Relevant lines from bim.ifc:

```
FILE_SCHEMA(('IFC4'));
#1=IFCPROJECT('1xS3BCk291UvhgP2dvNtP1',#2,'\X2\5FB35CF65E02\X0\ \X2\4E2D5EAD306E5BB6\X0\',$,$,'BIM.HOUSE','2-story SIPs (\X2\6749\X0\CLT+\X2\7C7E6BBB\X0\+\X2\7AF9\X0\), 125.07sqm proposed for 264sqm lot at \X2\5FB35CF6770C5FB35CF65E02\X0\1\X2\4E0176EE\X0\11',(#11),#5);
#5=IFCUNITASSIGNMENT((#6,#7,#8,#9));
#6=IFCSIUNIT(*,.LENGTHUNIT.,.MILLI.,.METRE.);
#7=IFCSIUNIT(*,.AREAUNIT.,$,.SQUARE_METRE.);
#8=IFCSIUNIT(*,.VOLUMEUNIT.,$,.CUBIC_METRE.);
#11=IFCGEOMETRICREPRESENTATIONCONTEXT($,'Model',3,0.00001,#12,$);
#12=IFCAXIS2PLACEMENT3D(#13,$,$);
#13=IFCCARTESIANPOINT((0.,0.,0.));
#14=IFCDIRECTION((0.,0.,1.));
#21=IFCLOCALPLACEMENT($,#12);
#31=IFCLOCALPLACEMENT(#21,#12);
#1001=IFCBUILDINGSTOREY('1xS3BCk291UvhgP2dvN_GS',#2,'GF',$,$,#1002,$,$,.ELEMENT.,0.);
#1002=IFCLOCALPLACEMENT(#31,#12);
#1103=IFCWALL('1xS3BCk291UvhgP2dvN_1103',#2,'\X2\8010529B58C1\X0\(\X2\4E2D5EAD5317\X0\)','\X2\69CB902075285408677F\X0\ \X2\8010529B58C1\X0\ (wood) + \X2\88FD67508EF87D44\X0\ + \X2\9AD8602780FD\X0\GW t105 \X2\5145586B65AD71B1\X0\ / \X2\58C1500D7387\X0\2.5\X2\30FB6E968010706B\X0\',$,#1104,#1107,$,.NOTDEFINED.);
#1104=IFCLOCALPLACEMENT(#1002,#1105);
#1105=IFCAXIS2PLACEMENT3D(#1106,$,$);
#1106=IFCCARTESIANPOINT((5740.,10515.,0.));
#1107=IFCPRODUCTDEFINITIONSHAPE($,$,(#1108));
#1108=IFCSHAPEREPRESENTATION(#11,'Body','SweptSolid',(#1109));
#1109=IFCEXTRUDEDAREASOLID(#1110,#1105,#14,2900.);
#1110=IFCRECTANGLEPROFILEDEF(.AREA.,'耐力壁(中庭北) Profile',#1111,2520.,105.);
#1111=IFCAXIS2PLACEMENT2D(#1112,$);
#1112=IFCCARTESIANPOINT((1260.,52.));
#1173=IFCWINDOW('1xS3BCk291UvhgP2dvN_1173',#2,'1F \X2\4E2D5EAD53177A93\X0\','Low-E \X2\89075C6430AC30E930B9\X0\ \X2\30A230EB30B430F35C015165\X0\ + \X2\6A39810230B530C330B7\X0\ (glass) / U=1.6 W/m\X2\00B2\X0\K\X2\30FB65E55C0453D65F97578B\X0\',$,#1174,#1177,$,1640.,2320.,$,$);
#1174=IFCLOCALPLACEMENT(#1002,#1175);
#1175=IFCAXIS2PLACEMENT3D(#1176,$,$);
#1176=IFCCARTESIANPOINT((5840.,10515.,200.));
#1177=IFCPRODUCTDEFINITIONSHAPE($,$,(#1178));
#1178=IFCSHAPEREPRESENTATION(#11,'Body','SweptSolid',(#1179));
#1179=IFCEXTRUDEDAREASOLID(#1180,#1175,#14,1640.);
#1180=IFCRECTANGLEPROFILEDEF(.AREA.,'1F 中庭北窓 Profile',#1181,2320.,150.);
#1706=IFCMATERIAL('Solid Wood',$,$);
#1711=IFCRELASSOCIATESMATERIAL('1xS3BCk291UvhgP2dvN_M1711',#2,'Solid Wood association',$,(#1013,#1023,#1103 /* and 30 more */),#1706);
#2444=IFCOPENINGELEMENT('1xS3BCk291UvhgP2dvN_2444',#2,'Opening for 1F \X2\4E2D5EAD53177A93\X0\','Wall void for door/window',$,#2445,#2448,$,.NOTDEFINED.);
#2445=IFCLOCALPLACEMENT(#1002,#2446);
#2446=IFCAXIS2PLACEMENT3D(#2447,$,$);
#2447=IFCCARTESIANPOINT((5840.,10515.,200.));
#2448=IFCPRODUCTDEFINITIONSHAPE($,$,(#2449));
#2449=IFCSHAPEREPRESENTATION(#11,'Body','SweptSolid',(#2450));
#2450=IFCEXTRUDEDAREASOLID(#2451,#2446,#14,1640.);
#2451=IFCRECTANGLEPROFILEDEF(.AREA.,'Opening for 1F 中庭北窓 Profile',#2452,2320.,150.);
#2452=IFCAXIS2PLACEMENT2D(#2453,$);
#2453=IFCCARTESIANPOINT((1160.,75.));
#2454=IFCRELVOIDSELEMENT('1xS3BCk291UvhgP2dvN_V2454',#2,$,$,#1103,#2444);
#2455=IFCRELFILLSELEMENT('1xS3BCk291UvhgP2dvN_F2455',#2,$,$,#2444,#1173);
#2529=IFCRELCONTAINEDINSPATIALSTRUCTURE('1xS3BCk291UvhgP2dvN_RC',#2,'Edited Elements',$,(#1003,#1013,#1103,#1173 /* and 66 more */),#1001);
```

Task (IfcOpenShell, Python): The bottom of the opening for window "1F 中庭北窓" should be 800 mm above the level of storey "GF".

```python
import numpy as np
import ifcopenshell
import ifcopenshell.api.geometry
import ifcopenshell.geom
import ifcopenshell.util.element
import ifcopenshell.util.placement
import ifcopenshell.util.shape
import ifcopenshell.util.unit

model = ifcopenshell.open("bim.ifc")
unit_scale = ifcopenshell.util.unit.calculate_unit_scale(model)

window = model.by_guid("1xS3BCk291UvhgP2dvN_1173")
opening = window.FillsVoids[0].RelatingOpeningElement
storey = ifcopenshell.util.element.get_container(window, ifc_class="IfcBuildingStorey")
level = ifcopenshell.util.placement.get_local_placement(storey.ObjectPlacement)[2, 3]

# The opening's origin need not be at the sill, so measure its lowest point.
shape = ifcopenshell.geom.create_shape(ifcopenshell.geom.settings(), opening)
bottom = ifcopenshell.util.shape.get_shape_bottom_elevation(shape, shape.geometry) / unit_scale
dz = level + 0.8 / unit_scale - bottom

shift = np.array([0.0, 0.0, dz])
# The window is not placed relative to its opening, so move both.
for product in (opening, window):
    matrix = ifcopenshell.util.placement.get_local_placement(product.ObjectPlacement)
    matrix[:3, 3] += shift
    ifcopenshell.api.geometry.edit_object_placement(model, product=product, matrix=matrix, is_si=False)

print(f"moved by {dz * unit_scale:+.3f} m")

model.write("bim_rev.ifc")
```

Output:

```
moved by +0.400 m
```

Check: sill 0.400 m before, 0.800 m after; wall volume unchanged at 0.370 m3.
